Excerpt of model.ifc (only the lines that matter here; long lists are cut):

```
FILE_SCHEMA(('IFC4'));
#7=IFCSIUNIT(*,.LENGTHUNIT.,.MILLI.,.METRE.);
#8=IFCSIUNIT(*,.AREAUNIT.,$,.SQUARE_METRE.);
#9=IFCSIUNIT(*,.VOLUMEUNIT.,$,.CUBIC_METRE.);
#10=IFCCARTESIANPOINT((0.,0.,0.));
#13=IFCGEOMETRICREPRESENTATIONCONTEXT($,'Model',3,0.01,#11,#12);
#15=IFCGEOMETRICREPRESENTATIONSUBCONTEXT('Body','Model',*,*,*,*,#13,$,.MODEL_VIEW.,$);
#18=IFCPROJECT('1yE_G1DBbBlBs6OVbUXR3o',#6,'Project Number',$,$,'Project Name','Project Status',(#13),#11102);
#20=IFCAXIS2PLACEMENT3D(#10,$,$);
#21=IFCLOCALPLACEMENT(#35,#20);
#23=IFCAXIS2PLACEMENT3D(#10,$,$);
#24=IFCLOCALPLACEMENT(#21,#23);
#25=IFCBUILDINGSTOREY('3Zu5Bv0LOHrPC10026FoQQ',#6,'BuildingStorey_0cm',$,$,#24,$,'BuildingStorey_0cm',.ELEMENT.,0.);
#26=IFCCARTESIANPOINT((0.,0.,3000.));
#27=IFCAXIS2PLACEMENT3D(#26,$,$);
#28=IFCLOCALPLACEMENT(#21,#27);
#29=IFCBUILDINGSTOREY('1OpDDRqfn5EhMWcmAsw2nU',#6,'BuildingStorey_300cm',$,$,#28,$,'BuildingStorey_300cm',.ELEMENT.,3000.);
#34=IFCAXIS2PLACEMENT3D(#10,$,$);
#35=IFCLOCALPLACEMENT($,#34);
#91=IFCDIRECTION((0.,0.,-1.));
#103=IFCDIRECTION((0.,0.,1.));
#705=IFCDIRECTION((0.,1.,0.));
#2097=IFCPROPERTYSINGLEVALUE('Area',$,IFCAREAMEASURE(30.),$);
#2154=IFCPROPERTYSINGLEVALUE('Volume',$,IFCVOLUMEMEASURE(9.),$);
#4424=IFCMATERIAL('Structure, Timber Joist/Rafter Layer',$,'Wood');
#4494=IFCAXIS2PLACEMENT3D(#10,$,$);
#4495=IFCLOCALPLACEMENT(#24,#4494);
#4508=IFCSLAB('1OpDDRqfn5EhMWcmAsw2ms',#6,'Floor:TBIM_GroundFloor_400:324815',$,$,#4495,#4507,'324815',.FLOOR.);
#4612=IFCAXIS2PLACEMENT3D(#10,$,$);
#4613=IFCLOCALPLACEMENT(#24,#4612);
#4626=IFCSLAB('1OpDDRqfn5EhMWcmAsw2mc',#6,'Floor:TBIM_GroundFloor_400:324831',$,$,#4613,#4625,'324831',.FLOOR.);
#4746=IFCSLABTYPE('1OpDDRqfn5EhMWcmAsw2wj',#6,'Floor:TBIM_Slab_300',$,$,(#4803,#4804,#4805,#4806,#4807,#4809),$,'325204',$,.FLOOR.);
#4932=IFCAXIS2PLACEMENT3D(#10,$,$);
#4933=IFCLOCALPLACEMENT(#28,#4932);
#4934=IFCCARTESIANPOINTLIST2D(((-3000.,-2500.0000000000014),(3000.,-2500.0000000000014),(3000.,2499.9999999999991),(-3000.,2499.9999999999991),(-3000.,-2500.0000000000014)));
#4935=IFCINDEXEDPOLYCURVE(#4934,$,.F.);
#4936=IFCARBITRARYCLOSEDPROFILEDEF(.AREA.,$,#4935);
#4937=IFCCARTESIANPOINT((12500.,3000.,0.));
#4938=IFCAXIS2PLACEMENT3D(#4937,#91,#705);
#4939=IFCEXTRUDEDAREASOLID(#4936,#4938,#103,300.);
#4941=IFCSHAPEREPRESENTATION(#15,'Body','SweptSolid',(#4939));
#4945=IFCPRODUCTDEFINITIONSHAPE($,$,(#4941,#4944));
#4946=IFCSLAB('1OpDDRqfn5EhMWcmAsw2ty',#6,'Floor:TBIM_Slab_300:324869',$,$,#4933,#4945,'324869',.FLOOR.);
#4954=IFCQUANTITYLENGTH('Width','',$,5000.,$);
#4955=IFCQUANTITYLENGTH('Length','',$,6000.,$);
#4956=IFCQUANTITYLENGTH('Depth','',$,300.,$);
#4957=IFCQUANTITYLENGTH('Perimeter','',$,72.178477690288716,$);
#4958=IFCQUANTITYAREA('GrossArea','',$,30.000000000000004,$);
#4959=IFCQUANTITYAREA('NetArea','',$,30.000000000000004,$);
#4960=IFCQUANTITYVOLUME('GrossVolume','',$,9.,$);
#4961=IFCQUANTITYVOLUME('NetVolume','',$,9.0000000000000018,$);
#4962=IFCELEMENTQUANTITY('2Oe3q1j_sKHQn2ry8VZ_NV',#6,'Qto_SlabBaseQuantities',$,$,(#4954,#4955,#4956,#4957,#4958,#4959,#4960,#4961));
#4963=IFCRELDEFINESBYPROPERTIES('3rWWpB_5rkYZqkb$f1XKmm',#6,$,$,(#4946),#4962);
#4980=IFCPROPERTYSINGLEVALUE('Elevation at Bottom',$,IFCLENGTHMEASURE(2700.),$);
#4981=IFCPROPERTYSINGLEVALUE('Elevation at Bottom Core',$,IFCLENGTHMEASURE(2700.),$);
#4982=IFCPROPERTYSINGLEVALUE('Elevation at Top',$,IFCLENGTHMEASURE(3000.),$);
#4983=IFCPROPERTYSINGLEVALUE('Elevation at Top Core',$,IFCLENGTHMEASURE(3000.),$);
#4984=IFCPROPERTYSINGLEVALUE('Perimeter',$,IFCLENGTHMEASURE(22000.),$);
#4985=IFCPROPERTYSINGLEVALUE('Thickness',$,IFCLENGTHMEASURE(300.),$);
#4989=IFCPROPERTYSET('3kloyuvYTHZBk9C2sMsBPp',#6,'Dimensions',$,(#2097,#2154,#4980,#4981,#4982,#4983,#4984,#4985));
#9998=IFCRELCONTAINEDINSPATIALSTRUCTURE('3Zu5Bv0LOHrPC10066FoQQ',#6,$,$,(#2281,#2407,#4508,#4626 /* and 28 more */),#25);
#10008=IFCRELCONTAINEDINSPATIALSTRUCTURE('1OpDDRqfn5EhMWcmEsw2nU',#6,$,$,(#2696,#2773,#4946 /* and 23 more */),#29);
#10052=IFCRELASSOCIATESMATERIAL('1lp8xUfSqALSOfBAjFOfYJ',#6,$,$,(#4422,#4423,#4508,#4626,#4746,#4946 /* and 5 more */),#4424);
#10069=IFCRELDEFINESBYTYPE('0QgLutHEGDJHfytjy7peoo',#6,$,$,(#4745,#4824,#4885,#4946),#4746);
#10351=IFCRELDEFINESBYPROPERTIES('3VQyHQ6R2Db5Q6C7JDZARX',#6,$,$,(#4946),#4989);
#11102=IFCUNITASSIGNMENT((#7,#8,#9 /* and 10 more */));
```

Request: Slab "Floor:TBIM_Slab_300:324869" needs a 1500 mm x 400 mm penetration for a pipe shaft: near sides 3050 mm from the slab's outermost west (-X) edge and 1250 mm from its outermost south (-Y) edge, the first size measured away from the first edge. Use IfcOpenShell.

```python
import numpy as np
import ifcopenshell
import ifcopenshell.api.feature
import ifcopenshell.api.geometry
import ifcopenshell.api.pset
import ifcopenshell.api.root
import ifcopenshell.geom
import ifcopenshell.util.element
import ifcopenshell.util.placement
import ifcopenshell.util.representation
import ifcopenshell.util.shape
import ifcopenshell.util.unit

model = ifcopenshell.open("model.ifc")
unit_scale = ifcopenshell.util.unit.calculate_unit_scale(model)
area_scale = ifcopenshell.util.unit.calculate_unit_scale(model, "AREAUNIT")
volume_scale = ifcopenshell.util.unit.calculate_unit_scale(model, "VOLUMEUNIT")
settings = ifcopenshell.geom.settings()


def volume(element):
    """Net volume in cubic metres, openings subtracted."""
    shape = ifcopenshell.geom.create_shape(settings, element)
    return ifcopenshell.util.shape.get_volume(shape.geometry)


slab = model.by_guid("1OpDDRqfn5EhMWcmAsw2ty")
before = volume(slab)

# Extent in the slab's own axes, in metres. The edges named are its -X and -Y sides.
slab_shape = ifcopenshell.geom.create_shape(settings, slab)
vertices = ifcopenshell.util.shape.get_vertices(slab_shape.geometry)
x_min, y_min, bottom = vertices.min(axis=0)
top = vertices[:, 2].max()

opening = ifcopenshell.api.root.create_entity(model, ifc_class="IfcOpeningElement", name="Pipe shaft opening", predefined_type="OPENING")
context = ifcopenshell.util.representation.get_context(model, "Model", "Body", "MODEL_VIEW")
width, depth = 1.5, 0.4
outline = [(0.0, 0.0), (width, 0.0), (width, depth), (0.0, depth), (0.0, 0.0)]
# Overshoot both faces by 50 mm so the cut is clean.
shape = ifcopenshell.api.geometry.add_slab_representation(
    model, context=context, depth=top - bottom + 0.1, polyline=outline
)
ifcopenshell.api.geometry.assign_representation(model, product=opening, representation=shape)

matrix = ifcopenshell.util.placement.get_local_placement(slab.ObjectPlacement)
matrix[:, 3] = matrix @ np.append(np.array([x_min + 3.05, y_min + 1.25, bottom - 0.05]) / unit_scale, 1.0)
ifcopenshell.api.geometry.edit_object_placement(model, product=opening, matrix=matrix, is_si=False)
ifcopenshell.api.feature.add_feature(model, feature=opening, element=slab)

after = volume(slab)

# Update the slab's stored quantities.
qto = model.by_id(ifcopenshell.util.element.get_pset(slab, "Qto_SlabBaseQuantities", should_inherit=False)["id"])
ifcopenshell.api.pset.edit_qto(model, qto=qto, properties={
    "NetArea": after / (top - bottom) / area_scale,
    "NetVolume": after / volume_scale,
})
pset = model.by_id(ifcopenshell.util.element.get_pset(slab, "Dimensions", should_inherit=False)["id"])
ifcopenshell.api.pset.edit_pset(model, pset=pset, properties={
    "Area": model.create_entity("IfcAreaMeasure", after / (top - bottom) / area_scale),
    "Volume": model.create_entity("IfcVolumeMeasure", after / volume_scale),
})

print(f"slab volume {before:.3f} -> {after:.3f} m3")

model.write("model_rev.ifc")
```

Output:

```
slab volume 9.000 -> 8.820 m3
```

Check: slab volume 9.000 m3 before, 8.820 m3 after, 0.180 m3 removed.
